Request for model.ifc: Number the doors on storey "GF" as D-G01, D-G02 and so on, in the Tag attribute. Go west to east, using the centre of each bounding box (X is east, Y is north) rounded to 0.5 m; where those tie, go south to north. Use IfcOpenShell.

First a look at what the model holds.

```python
import ifcopenshell
import ifcopenshell.util.element
import ifcopenshell.util.placement

model = ifcopenshell.open("model.ifc")
print(model.schema)
storey = next(s for s in model.by_type("IfcBuildingStorey") if s.Name == "GF")
doors = [e for e in ifcopenshell.util.element.get_decomposition(storey) if e.is_a("IfcDoor")]
for e in sorted(doors, key=lambda e: e.id()):
    origin = ifcopenshell.util.placement.get_local_placement(e.ObjectPlacement)[:3, 3]
    print(e.id(), e.Tag, e.Name, origin.round(2) + 0.0, sep=" | ")
```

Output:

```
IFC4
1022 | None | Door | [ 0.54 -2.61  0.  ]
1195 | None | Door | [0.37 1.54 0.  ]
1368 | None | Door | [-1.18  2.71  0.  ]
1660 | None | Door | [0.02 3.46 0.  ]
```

```python
import ifcopenshell
import ifcopenshell.geom
import ifcopenshell.util.element
import ifcopenshell.util.shape

model = ifcopenshell.open("model.ifc")
settings = ifcopenshell.geom.settings()
settings.set("use-world-coords", True)


def centre(element):
    shape = ifcopenshell.geom.create_shape(settings, element)
    return ifcopenshell.util.shape.get_bbox_centroid(shape.geometry)


storey = next(s for s in model.by_type("IfcBuildingStorey") if s.Name == "GF")
doors = [e for e in ifcopenshell.util.element.get_decomposition(storey) if e.is_a("IfcDoor")]

# Insertion points can sit at a corner or the storey origin, so sort by the geometry (in metres).
centres = {e: centre(e) for e in doors}
doors.sort(key=lambda e: (round(centres[e][0] / 0.5), centres[e][1]))

for i, e in enumerate(doors, start=1):
    number = f"D-G{i:02d}"
    e.Tag = number
    print(e.id(), number)

model.write("model_rev.ifc")
```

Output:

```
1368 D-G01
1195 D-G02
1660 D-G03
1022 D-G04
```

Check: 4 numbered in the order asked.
